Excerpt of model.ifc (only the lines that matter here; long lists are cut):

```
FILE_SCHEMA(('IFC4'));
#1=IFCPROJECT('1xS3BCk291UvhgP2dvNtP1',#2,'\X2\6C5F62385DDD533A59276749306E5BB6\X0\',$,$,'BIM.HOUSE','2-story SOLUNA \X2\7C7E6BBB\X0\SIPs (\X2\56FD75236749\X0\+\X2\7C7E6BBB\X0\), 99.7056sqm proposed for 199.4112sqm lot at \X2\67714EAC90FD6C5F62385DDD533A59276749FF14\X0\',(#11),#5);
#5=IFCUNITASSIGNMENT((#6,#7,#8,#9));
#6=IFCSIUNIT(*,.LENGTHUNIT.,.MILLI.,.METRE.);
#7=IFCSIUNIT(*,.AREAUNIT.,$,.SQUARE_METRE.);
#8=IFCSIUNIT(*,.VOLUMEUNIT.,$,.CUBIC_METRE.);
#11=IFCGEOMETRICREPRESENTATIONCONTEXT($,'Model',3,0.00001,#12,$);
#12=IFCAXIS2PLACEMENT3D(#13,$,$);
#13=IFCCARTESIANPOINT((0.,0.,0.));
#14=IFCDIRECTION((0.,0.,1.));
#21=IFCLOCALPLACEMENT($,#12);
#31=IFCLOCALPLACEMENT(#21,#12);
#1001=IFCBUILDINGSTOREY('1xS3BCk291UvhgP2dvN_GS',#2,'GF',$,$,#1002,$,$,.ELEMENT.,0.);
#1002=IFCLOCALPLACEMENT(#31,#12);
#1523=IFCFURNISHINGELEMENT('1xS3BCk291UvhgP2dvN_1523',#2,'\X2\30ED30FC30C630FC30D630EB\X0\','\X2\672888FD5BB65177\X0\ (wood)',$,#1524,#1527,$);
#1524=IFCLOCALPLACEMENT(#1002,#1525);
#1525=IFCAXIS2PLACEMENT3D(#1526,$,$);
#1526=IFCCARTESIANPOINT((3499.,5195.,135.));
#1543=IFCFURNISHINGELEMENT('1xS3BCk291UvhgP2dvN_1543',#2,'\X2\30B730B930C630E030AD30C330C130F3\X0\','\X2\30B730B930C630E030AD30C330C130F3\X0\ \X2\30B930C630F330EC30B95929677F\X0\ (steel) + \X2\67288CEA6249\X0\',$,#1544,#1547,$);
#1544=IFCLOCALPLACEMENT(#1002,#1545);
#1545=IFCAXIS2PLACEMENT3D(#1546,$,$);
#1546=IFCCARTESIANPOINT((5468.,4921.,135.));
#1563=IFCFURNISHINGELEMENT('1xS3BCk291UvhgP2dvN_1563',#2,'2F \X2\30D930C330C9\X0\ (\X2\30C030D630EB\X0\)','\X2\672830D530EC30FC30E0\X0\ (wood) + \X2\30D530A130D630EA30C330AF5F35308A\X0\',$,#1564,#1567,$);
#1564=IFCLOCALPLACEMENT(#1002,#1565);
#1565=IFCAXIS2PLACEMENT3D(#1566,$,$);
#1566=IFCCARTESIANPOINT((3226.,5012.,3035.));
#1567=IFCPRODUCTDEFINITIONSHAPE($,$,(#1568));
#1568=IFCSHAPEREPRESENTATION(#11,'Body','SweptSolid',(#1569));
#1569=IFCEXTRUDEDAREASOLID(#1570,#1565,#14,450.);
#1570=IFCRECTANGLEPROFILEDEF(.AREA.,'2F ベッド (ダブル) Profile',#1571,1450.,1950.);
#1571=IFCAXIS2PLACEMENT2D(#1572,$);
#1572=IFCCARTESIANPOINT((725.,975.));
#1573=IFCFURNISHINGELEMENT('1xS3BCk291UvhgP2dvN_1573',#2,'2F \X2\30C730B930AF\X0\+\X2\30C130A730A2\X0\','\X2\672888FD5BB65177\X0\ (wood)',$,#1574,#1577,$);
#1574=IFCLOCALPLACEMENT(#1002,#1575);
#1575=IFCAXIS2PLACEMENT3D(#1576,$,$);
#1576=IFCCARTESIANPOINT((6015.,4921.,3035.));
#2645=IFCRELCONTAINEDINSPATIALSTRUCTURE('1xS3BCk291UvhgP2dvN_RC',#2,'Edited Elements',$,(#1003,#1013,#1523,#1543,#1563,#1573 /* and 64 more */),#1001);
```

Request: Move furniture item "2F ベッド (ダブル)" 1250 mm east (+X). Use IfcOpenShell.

```python
import ifcopenshell
import ifcopenshell.api.geometry
import ifcopenshell.util.placement
import ifcopenshell.util.unit

model = ifcopenshell.open("model.ifc")
unit_scale = ifcopenshell.util.unit.calculate_unit_scale(model)

item = model.by_guid("1xS3BCk291UvhgP2dvN_1563")
matrix = ifcopenshell.util.placement.get_local_placement(item.ObjectPlacement)
matrix[0, 3] += 1.25 / unit_scale
ifcopenshell.api.geometry.edit_object_placement(model, product=item, matrix=matrix, is_si=False)

print(ifcopenshell.util.placement.get_local_placement(item.ObjectPlacement).round(3) + 0.0)

model.write("model-out.ifc")
```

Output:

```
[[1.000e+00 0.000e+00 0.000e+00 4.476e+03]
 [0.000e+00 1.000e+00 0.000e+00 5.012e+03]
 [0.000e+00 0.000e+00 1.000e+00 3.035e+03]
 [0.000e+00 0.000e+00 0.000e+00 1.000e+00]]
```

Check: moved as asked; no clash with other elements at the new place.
